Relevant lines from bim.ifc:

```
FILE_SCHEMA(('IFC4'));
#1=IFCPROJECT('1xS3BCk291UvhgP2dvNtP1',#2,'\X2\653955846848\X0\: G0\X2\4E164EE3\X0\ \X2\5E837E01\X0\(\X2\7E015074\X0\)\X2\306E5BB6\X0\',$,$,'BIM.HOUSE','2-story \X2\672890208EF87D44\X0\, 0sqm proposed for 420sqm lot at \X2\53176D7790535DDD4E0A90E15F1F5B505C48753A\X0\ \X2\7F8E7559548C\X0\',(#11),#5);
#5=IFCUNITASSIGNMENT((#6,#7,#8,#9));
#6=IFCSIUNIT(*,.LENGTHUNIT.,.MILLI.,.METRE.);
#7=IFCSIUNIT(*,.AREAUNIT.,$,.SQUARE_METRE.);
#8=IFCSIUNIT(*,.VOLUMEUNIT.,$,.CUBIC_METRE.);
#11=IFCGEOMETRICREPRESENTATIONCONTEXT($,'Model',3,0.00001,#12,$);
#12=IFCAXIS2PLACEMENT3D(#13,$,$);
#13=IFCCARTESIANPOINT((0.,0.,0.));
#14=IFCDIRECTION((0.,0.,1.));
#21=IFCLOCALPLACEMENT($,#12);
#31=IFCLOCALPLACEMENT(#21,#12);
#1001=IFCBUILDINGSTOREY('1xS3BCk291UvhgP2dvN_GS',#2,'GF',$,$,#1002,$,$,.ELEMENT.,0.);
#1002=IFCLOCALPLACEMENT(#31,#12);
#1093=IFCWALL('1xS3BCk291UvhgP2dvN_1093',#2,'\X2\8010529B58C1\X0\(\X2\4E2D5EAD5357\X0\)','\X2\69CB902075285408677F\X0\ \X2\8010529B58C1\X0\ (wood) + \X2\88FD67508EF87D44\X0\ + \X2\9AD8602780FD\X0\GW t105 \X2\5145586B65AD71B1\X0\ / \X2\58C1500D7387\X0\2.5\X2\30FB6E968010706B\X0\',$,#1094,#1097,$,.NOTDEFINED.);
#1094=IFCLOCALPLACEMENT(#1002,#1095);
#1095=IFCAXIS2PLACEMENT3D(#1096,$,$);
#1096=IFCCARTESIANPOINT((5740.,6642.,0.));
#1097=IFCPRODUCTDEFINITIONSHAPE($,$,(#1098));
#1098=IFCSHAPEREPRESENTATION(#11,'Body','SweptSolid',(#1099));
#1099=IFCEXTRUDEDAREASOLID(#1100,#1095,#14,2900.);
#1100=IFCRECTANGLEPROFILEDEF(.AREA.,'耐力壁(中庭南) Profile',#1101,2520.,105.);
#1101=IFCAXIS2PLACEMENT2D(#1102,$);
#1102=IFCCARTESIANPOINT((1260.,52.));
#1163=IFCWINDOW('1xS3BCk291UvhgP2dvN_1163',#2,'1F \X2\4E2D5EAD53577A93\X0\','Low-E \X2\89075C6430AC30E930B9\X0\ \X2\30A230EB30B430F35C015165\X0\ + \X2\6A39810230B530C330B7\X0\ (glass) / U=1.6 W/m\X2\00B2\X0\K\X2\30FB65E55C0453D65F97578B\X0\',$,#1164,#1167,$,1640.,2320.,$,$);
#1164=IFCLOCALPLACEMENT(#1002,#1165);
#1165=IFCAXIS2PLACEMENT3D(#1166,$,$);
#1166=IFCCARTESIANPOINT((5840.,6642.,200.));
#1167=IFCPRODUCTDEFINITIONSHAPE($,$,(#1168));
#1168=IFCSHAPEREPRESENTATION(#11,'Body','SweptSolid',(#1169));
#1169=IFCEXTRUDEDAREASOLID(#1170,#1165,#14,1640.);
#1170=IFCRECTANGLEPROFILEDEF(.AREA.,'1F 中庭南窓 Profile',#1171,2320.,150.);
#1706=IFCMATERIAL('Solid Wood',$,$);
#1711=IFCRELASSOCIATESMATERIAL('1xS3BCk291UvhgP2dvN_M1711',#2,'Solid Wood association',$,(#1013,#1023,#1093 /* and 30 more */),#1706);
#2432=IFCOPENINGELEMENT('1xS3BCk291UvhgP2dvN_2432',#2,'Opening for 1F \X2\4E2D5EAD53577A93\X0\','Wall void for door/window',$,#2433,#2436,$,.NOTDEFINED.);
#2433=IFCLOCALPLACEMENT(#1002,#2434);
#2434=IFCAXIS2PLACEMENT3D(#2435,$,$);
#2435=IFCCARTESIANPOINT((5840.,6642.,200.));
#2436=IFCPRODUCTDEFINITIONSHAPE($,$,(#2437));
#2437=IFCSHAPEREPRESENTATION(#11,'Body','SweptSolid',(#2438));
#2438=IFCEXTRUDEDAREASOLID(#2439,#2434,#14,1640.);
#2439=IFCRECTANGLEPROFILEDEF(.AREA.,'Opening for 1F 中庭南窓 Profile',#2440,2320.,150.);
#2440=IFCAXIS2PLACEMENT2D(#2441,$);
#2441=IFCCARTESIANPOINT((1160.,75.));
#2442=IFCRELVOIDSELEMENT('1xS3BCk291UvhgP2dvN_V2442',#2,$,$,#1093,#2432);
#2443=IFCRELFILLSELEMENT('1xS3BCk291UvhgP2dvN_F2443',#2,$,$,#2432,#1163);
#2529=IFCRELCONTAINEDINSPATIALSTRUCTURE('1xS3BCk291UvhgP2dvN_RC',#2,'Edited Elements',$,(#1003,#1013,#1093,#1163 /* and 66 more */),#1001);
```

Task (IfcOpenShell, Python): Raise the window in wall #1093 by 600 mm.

```python
import numpy as np
import ifcopenshell
import ifcopenshell.api.geometry
import ifcopenshell.util.placement
import ifcopenshell.util.unit

model = ifcopenshell.open("bim.ifc")
unit_scale = ifcopenshell.util.unit.calculate_unit_scale(model)

window = model.by_id(1163)
opening = window.FillsVoids[0].RelatingOpeningElement
dz = 0.6 / unit_scale

shift = np.array([0.0, 0.0, dz])
# The window is not placed relative to its opening, so move both.
for product in (opening, window):
    matrix = ifcopenshell.util.placement.get_local_placement(product.ObjectPlacement)
    matrix[:3, 3] += shift
    ifcopenshell.api.geometry.edit_object_placement(model, product=product, matrix=matrix, is_si=False)

print(f"moved by {dz * unit_scale:+.3f} m")

model.write("bim_rev.ifc")
```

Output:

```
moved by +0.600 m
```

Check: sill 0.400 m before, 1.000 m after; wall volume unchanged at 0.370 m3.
